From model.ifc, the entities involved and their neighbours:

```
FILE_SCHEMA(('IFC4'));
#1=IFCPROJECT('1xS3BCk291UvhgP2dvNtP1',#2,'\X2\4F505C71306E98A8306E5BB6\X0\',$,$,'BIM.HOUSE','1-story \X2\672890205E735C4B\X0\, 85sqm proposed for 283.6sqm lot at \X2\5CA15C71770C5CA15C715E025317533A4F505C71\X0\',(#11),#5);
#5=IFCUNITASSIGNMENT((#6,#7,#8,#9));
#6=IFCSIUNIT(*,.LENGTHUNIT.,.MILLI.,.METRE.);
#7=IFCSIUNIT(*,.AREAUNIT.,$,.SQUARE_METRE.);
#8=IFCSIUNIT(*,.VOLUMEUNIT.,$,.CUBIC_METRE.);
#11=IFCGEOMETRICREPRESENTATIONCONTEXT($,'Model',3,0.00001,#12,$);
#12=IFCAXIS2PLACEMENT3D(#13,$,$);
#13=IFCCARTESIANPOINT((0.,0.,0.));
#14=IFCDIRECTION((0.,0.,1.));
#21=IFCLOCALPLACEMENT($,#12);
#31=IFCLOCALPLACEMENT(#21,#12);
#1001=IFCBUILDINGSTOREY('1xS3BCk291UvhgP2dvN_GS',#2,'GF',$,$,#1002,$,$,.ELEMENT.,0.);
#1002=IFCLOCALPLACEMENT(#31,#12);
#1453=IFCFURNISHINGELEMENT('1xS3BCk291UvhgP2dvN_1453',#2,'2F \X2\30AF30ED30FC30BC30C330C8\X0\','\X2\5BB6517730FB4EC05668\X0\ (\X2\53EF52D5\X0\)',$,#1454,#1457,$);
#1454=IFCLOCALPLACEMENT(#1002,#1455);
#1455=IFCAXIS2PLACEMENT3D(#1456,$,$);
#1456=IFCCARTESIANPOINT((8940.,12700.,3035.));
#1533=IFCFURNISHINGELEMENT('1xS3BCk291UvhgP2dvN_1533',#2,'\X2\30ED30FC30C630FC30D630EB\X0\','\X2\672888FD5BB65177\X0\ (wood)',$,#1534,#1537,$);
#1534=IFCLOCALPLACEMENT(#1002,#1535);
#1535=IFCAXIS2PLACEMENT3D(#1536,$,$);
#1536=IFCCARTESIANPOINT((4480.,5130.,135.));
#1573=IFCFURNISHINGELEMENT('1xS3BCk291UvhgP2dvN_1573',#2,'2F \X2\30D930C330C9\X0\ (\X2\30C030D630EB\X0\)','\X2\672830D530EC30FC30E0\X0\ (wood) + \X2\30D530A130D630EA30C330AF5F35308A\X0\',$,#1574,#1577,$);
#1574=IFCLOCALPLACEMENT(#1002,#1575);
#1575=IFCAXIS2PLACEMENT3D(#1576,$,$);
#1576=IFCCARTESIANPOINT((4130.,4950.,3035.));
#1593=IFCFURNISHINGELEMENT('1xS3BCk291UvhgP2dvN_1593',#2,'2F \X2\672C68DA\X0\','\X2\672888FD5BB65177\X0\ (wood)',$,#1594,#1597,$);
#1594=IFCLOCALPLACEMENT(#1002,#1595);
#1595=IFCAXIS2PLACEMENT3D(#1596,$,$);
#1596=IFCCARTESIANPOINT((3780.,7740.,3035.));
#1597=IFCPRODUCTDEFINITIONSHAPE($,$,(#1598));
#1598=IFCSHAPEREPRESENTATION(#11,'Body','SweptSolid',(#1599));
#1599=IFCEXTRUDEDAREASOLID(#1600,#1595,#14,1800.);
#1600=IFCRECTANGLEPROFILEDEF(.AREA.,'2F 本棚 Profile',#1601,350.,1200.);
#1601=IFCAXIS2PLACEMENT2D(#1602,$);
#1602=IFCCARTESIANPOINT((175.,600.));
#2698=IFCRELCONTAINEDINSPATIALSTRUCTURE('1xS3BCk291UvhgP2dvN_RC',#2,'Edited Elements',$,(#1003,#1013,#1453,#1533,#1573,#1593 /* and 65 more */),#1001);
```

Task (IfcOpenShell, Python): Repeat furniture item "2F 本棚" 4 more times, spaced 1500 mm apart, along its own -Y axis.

```python
import ifcopenshell
import ifcopenshell.api.geometry
import ifcopenshell.api.root
import ifcopenshell.util.element
import ifcopenshell.util.placement

model = ifcopenshell.open("model.ifc")


def reuse_history(source, copy):
    """copy_class also copies each property set's owner history, people and application; keep the originals."""
    for rel in copy.IsDefinedBy:
        if rel.is_a("IfcRelDefinesByProperties") and (history := rel.RelatingPropertyDefinition.OwnerHistory):
            rel.RelatingPropertyDefinition.OwnerHistory = source.OwnerHistory
            ifcopenshell.util.element.remove_deep2(model, history)


source = model.by_id(1593)
base = ifcopenshell.util.placement.get_local_placement(source.ObjectPlacement)
step = -base[:3, 1] * 1500.0

for i in range(1, 5):
    copy = ifcopenshell.api.root.copy_class(model, product=source)
    copy.Representation = ifcopenshell.util.element.copy_deep(
        model, source.Representation, exclude=["IfcGeometricRepresentationContext", "IfcRepresentationMap"]
    )
    reuse_history(source, copy)
    matrix = base.copy()
    matrix[:3, 3] += i * step
    print("added at", matrix[:3, 3].round(3) + 0.0)
    ifcopenshell.api.geometry.edit_object_placement(model, product=copy, matrix=matrix, is_si=False)

model.write("model-out.ifc")
```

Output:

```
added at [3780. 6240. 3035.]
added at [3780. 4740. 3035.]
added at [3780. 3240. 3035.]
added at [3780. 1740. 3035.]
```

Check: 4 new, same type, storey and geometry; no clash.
